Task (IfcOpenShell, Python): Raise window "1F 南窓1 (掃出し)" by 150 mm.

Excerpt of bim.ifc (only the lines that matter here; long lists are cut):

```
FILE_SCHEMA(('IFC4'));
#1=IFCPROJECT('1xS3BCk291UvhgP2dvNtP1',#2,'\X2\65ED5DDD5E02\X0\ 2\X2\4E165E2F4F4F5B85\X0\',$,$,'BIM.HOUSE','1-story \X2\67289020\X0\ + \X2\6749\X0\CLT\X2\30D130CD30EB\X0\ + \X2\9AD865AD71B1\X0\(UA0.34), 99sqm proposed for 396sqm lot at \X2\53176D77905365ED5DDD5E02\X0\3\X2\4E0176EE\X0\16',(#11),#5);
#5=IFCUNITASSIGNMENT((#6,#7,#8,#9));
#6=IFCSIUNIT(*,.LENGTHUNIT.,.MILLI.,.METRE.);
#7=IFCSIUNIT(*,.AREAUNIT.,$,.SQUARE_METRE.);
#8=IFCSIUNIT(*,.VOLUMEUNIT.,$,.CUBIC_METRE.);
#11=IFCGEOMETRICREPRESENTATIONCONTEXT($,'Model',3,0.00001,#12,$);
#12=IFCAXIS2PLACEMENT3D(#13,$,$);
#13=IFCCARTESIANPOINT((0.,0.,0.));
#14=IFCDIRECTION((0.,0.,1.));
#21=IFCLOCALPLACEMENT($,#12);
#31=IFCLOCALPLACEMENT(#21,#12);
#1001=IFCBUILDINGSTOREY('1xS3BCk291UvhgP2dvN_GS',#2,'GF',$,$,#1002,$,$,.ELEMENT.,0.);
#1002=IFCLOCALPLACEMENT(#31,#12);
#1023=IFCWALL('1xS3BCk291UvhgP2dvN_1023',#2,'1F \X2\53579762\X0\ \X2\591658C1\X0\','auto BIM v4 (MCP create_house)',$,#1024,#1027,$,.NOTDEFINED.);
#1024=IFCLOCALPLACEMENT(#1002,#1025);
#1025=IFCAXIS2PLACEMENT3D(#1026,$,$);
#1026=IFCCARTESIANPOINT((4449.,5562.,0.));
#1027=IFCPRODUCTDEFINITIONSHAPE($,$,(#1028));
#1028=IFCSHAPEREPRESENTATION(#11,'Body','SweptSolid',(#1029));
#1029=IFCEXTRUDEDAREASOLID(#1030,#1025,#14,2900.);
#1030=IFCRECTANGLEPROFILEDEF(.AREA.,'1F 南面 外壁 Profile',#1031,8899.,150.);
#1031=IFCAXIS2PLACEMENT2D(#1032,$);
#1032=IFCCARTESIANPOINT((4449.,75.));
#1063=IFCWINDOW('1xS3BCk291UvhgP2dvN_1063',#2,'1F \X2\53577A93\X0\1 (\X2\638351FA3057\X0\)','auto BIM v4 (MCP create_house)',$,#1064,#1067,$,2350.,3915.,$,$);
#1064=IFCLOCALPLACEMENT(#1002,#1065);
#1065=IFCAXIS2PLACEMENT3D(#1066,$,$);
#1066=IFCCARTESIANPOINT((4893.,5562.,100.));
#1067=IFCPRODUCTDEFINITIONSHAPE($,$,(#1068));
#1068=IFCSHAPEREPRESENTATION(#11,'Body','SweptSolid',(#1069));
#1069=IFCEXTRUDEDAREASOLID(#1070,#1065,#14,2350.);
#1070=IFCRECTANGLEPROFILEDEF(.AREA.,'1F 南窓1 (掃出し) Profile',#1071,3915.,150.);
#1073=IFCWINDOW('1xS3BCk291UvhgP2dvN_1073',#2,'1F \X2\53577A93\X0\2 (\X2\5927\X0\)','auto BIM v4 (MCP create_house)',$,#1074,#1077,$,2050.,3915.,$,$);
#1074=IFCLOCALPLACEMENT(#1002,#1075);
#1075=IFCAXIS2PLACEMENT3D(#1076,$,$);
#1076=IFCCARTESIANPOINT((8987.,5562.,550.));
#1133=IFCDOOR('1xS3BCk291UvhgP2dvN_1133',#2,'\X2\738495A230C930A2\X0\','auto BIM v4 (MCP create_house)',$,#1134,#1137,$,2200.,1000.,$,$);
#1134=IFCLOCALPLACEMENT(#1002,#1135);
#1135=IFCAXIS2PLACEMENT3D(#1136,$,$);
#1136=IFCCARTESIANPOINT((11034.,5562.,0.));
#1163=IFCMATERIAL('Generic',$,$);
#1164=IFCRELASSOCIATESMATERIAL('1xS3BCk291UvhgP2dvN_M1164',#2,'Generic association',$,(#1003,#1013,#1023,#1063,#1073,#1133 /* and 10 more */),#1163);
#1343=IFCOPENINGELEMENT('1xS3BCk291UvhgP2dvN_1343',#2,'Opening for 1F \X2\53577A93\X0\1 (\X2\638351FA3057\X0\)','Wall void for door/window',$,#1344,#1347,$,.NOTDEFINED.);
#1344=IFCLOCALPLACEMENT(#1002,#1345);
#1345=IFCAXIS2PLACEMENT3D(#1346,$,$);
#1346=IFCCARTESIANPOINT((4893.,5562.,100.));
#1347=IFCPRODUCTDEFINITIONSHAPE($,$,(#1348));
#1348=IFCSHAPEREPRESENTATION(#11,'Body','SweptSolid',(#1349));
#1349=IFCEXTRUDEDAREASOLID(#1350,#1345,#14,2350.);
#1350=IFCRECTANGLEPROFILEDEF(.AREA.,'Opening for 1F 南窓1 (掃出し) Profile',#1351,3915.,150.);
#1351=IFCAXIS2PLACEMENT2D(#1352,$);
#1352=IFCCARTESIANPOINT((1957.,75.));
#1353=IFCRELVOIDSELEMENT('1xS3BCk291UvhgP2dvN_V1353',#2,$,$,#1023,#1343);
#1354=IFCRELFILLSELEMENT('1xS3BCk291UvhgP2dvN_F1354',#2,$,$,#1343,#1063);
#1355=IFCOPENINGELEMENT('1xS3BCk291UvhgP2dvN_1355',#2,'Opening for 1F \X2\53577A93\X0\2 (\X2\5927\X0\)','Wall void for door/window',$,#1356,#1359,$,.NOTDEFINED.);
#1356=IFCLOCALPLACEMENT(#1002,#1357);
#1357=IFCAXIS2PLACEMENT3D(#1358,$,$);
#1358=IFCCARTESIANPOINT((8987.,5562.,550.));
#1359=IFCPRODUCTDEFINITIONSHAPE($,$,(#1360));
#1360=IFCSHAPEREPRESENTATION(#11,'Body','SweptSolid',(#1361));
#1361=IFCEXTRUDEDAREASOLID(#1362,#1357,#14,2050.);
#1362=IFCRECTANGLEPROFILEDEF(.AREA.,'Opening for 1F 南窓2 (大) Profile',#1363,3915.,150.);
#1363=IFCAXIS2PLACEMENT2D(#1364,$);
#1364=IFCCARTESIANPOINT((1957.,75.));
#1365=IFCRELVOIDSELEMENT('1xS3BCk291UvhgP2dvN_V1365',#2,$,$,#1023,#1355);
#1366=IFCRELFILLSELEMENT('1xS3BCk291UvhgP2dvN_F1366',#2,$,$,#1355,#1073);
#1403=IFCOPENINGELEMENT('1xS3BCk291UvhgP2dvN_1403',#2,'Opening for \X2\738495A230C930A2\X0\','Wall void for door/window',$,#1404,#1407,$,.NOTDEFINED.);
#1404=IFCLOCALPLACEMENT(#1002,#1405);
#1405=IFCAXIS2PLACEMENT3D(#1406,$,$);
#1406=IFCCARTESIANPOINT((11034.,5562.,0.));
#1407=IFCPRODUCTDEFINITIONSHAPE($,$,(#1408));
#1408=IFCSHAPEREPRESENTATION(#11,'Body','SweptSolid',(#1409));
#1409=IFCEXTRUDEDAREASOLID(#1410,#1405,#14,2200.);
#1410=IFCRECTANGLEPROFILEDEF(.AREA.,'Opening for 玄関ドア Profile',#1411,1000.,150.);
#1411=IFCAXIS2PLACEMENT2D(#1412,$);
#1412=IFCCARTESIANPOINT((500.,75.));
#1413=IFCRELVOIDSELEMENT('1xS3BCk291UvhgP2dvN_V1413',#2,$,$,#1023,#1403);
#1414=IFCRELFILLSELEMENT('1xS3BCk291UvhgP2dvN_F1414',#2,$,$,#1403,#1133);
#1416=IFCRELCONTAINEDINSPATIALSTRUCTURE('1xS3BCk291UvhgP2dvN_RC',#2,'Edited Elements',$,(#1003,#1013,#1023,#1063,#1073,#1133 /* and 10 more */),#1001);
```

```python
import numpy as np
import ifcopenshell
import ifcopenshell.api.geometry
import ifcopenshell.util.placement
import ifcopenshell.util.unit

model = ifcopenshell.open("bim.ifc")
unit_scale = ifcopenshell.util.unit.calculate_unit_scale(model)

window = model.by_guid("1xS3BCk291UvhgP2dvN_1063")
opening = window.FillsVoids[0].RelatingOpeningElement
dz = 0.15 / unit_scale

shift = np.array([0.0, 0.0, dz])
# The window is not placed relative to its opening, so move both.
for product in (opening, window):
    matrix = ifcopenshell.util.placement.get_local_placement(product.ObjectPlacement)
    matrix[:3, 3] += shift
    ifcopenshell.api.geometry.edit_object_placement(model, product=product, matrix=matrix, is_si=False)

print(f"moved by {dz * unit_scale:+.3f} m")

model.write("bim-out.ifc")
```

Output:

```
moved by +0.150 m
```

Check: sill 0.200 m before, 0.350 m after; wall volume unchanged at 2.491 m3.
